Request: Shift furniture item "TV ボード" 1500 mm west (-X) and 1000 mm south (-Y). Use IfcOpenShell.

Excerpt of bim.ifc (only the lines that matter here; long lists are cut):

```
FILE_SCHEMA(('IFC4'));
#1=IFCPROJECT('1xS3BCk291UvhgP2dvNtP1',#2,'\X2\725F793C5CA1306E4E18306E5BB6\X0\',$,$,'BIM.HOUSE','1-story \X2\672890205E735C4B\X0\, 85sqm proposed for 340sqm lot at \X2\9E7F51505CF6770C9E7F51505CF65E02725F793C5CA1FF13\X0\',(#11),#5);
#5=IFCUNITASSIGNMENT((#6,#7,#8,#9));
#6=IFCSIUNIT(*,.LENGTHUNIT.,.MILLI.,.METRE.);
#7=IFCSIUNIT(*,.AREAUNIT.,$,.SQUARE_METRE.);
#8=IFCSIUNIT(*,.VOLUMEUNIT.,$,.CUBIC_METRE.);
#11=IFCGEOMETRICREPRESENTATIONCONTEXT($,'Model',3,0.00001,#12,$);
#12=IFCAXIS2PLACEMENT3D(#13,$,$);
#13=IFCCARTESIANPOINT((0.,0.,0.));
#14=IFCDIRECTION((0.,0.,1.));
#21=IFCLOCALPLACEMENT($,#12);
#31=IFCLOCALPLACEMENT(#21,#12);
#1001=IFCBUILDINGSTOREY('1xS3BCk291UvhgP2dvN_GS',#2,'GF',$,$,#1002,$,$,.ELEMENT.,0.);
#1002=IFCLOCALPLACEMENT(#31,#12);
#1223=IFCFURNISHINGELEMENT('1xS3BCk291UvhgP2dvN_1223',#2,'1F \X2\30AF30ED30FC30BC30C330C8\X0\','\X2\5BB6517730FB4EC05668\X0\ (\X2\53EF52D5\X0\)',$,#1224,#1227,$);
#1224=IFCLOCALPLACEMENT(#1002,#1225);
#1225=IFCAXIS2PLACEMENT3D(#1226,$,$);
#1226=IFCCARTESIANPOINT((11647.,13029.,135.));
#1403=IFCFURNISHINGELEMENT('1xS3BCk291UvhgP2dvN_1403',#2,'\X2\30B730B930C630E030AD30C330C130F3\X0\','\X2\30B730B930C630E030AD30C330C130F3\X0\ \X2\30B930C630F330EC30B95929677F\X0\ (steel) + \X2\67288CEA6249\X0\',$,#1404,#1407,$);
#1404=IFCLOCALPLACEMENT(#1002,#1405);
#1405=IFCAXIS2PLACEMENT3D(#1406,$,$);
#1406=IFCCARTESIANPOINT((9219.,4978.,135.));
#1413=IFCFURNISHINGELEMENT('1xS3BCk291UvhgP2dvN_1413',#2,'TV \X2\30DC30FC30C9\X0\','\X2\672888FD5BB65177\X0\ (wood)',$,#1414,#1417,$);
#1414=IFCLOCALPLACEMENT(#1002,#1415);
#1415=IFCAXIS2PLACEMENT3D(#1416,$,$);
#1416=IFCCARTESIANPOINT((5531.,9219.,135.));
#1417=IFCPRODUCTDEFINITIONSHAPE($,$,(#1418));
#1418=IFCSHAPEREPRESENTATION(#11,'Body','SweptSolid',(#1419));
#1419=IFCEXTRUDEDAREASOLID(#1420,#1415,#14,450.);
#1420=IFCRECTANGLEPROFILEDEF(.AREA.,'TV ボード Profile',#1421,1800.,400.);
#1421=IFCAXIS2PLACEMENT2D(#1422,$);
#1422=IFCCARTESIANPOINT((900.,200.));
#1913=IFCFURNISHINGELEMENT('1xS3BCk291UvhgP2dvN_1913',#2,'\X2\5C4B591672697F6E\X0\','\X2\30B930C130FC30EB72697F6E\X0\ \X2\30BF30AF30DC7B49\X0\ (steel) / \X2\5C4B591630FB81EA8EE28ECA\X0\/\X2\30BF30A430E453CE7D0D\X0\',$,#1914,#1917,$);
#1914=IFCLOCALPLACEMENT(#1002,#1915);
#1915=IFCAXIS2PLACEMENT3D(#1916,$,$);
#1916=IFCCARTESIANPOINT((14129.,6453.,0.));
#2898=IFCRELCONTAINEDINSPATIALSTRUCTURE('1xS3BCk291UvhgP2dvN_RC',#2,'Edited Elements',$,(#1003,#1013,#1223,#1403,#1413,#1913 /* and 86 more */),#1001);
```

```python
import ifcopenshell
import ifcopenshell.api.geometry
import ifcopenshell.util.placement

model = ifcopenshell.open("bim.ifc")

item = model.by_guid("1xS3BCk291UvhgP2dvN_1413")
matrix = ifcopenshell.util.placement.get_local_placement(item.ObjectPlacement)
matrix[0, 3] -= 1500.0
matrix[1, 3] -= 1000.0
ifcopenshell.api.geometry.edit_object_placement(model, product=item, matrix=matrix, is_si=False)

print(ifcopenshell.util.placement.get_local_placement(item.ObjectPlacement).round(3) + 0.0)

model.write("bim_edited.ifc")
```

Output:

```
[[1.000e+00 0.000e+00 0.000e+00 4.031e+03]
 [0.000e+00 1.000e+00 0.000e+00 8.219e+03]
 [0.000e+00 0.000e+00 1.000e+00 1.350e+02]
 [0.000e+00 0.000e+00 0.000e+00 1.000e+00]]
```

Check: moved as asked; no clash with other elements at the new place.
